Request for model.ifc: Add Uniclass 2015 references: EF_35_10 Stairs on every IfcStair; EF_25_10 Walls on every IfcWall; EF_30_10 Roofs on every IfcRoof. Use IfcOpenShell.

First a look at what the model holds.

```python
import ifcopenshell

model = ifcopenshell.open("model.ifc")
print(model.schema)
print("classifications:", [c.Name for c in model.by_type("IfcClassification")])
for ifc_class in ("IfcDoor", "IfcRoof", "IfcStair", "IfcWall", "IfcWindow"):
    print(ifc_class, len(model.by_type(ifc_class)))
```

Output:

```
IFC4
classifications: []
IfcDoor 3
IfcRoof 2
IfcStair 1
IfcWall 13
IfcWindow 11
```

```python
import ifcopenshell
import ifcopenshell.api.classification

model = ifcopenshell.open("model.ifc")

system = ifcopenshell.api.classification.add_classification(model, classification="Uniclass 2015")

codes = {
    "IfcStair": ("EF_35_10", "Stairs"),
    "IfcWall": ("EF_25_10", "Walls"),
    "IfcRoof": ("EF_30_10", "Roofs"),
}
for ifc_class, (code, name) in codes.items():
    products = model.by_type(ifc_class)
    ifcopenshell.api.classification.add_reference(
        model, products=products, classification=system, identification=code, name=name
    )
    print(code, len(products))

model.write("model_rev.ifc")
```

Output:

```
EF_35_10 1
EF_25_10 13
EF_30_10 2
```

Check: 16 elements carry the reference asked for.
